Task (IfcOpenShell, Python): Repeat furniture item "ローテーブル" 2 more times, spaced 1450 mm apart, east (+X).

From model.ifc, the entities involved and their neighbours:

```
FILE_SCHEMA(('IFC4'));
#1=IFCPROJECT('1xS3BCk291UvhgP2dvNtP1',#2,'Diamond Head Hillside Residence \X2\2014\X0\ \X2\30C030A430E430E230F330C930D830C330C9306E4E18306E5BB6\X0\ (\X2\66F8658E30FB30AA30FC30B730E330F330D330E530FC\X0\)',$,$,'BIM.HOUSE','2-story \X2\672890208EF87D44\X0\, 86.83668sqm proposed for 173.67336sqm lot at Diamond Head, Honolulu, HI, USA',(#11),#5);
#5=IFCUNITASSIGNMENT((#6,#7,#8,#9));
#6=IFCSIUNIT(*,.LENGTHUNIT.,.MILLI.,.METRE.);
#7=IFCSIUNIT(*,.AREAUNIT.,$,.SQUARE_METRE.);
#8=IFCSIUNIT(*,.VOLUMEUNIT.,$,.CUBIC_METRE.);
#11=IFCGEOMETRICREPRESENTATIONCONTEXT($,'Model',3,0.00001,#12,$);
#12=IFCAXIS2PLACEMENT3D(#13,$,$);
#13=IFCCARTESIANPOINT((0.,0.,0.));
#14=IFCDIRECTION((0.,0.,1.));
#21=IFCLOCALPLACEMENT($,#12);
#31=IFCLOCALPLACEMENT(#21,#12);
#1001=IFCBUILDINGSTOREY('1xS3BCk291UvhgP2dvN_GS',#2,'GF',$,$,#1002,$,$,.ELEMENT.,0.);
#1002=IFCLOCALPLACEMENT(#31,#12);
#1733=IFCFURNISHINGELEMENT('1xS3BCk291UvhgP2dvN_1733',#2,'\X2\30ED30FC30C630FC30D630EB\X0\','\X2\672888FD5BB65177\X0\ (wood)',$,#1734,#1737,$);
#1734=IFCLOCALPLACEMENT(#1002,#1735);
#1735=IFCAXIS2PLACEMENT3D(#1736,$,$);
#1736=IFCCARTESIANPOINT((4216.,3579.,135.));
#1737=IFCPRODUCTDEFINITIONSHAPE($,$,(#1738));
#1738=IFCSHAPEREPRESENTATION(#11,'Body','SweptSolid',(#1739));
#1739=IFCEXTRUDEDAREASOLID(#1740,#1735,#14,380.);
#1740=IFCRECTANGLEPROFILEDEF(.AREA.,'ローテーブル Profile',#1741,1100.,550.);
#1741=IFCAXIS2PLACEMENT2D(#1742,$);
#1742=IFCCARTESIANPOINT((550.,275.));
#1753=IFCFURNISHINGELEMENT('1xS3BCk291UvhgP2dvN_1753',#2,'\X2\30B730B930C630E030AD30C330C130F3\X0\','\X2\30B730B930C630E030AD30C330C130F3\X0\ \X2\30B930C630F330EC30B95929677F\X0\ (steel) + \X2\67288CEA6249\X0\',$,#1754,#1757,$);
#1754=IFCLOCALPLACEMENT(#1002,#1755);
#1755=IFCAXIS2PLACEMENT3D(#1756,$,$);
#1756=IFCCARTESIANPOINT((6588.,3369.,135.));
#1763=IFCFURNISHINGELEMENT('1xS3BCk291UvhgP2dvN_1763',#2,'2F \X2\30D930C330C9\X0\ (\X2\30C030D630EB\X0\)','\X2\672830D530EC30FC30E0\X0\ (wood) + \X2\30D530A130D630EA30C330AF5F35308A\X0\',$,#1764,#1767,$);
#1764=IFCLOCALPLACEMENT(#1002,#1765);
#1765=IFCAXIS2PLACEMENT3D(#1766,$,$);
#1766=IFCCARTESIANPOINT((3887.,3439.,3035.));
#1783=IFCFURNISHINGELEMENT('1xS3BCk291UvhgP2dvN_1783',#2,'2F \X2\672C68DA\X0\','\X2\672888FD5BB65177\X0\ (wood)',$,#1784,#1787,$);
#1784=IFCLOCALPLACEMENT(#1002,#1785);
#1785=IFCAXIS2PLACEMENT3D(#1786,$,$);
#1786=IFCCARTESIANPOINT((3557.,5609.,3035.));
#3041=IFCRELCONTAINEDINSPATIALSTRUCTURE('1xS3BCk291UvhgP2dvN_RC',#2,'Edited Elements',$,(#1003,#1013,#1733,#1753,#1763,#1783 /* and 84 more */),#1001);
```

```python
import numpy as np
import ifcopenshell
import ifcopenshell.api.geometry
import ifcopenshell.api.root
import ifcopenshell.util.element
import ifcopenshell.util.placement
import ifcopenshell.util.unit

model = ifcopenshell.open("model.ifc")
unit_scale = ifcopenshell.util.unit.calculate_unit_scale(model)


def reuse_history(source, copy):
    """copy_class also copies each property set's owner history, people and application; keep the originals."""
    for rel in copy.IsDefinedBy:
        if rel.is_a("IfcRelDefinesByProperties") and (history := rel.RelatingPropertyDefinition.OwnerHistory):
            rel.RelatingPropertyDefinition.OwnerHistory = source.OwnerHistory
            ifcopenshell.util.element.remove_deep2(model, history)


source = model.by_guid("1xS3BCk291UvhgP2dvN_1733")
base = ifcopenshell.util.placement.get_local_placement(source.ObjectPlacement)
step = np.array([1.0, 0.0, 0.0]) * 1.45 / unit_scale

for i in range(1, 3):
    copy = ifcopenshell.api.root.copy_class(model, product=source)
    copy.Representation = ifcopenshell.util.element.copy_deep(
        model, source.Representation, exclude=["IfcGeometricRepresentationContext", "IfcRepresentationMap"]
    )
    reuse_history(source, copy)
    matrix = base.copy()
    matrix[:3, 3] += i * step
    print("added at", matrix[:3, 3].round(3) + 0.0)
    ifcopenshell.api.geometry.edit_object_placement(model, product=copy, matrix=matrix, is_si=False)

model.write("model-out.ifc")
```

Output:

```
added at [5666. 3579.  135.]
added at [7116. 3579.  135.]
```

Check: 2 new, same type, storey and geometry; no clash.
